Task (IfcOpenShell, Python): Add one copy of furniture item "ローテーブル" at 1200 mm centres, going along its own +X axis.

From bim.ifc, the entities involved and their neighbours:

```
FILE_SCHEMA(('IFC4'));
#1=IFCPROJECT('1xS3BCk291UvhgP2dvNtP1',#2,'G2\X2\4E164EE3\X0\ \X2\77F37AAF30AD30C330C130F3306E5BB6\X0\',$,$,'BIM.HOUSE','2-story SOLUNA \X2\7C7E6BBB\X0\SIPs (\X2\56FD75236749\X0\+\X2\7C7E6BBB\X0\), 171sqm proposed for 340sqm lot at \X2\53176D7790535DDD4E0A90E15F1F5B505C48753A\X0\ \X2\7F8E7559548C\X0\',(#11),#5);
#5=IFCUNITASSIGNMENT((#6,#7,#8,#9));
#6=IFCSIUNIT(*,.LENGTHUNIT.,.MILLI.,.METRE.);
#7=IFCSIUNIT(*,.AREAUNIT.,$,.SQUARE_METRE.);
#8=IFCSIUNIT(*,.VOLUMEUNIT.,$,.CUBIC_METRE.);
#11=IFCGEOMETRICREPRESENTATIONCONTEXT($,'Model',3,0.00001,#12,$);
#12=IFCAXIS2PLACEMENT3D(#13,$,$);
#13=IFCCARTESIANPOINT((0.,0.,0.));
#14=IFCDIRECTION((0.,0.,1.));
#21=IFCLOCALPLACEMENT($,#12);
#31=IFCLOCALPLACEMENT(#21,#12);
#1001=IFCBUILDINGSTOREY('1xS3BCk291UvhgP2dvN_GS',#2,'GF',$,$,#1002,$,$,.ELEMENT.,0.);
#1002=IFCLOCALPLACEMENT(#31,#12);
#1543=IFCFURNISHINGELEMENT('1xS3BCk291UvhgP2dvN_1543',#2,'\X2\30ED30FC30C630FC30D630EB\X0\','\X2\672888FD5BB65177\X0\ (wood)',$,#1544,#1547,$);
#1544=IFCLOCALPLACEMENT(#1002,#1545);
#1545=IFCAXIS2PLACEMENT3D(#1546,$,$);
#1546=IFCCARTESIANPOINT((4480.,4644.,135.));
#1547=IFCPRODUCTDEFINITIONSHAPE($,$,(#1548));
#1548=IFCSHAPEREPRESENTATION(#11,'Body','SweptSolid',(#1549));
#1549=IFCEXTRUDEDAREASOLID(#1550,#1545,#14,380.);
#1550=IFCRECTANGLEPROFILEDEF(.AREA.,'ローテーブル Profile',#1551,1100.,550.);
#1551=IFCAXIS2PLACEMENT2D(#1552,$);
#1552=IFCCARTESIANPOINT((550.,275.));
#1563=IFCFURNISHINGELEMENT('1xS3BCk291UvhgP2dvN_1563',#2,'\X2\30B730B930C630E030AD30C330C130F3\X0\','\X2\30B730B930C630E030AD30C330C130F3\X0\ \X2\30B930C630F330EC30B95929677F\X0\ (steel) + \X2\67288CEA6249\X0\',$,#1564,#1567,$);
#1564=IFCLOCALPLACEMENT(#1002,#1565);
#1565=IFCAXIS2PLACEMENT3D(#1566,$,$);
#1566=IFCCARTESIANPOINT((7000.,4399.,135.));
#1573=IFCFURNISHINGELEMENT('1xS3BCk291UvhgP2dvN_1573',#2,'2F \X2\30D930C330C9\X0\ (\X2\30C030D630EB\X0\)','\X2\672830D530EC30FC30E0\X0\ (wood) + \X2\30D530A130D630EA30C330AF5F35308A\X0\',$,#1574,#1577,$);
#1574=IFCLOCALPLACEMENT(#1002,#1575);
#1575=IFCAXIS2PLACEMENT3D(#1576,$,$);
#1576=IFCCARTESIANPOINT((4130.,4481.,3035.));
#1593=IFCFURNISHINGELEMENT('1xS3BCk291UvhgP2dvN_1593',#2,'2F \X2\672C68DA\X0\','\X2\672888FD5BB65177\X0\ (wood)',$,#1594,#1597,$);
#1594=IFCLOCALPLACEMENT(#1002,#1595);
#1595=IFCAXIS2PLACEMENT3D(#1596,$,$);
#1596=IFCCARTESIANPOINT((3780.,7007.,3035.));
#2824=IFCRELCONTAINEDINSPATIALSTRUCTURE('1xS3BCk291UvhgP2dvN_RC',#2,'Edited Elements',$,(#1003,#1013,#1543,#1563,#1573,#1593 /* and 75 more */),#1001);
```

```python
import ifcopenshell
import ifcopenshell.api.geometry
import ifcopenshell.api.root
import ifcopenshell.util.element
import ifcopenshell.util.placement

model = ifcopenshell.open("bim.ifc")


def reuse_history(source, copy):
    """copy_class also copies each property set's owner history, people and application; keep the originals."""
    for rel in copy.IsDefinedBy:
        if rel.is_a("IfcRelDefinesByProperties") and (history := rel.RelatingPropertyDefinition.OwnerHistory):
            rel.RelatingPropertyDefinition.OwnerHistory = source.OwnerHistory
            ifcopenshell.util.element.remove_deep2(model, history)


source = model.by_guid("1xS3BCk291UvhgP2dvN_1543")
base = ifcopenshell.util.placement.get_local_placement(source.ObjectPlacement)
step = base[:3, 0] * 1200.0

for i in range(1, 2):
    copy = ifcopenshell.api.root.copy_class(model, product=source)
    copy.Representation = ifcopenshell.util.element.copy_deep(
        model, source.Representation, exclude=["IfcGeometricRepresentationContext", "IfcRepresentationMap"]
    )
    reuse_history(source, copy)
    matrix = base.copy()
    matrix[:3, 3] += i * step
    print("added at", matrix[:3, 3].round(3) + 0.0)
    ifcopenshell.api.geometry.edit_object_placement(model, product=copy, matrix=matrix, is_si=False)

model.write("bim_rev.ifc")
```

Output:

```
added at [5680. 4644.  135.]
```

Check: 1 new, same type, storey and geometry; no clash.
